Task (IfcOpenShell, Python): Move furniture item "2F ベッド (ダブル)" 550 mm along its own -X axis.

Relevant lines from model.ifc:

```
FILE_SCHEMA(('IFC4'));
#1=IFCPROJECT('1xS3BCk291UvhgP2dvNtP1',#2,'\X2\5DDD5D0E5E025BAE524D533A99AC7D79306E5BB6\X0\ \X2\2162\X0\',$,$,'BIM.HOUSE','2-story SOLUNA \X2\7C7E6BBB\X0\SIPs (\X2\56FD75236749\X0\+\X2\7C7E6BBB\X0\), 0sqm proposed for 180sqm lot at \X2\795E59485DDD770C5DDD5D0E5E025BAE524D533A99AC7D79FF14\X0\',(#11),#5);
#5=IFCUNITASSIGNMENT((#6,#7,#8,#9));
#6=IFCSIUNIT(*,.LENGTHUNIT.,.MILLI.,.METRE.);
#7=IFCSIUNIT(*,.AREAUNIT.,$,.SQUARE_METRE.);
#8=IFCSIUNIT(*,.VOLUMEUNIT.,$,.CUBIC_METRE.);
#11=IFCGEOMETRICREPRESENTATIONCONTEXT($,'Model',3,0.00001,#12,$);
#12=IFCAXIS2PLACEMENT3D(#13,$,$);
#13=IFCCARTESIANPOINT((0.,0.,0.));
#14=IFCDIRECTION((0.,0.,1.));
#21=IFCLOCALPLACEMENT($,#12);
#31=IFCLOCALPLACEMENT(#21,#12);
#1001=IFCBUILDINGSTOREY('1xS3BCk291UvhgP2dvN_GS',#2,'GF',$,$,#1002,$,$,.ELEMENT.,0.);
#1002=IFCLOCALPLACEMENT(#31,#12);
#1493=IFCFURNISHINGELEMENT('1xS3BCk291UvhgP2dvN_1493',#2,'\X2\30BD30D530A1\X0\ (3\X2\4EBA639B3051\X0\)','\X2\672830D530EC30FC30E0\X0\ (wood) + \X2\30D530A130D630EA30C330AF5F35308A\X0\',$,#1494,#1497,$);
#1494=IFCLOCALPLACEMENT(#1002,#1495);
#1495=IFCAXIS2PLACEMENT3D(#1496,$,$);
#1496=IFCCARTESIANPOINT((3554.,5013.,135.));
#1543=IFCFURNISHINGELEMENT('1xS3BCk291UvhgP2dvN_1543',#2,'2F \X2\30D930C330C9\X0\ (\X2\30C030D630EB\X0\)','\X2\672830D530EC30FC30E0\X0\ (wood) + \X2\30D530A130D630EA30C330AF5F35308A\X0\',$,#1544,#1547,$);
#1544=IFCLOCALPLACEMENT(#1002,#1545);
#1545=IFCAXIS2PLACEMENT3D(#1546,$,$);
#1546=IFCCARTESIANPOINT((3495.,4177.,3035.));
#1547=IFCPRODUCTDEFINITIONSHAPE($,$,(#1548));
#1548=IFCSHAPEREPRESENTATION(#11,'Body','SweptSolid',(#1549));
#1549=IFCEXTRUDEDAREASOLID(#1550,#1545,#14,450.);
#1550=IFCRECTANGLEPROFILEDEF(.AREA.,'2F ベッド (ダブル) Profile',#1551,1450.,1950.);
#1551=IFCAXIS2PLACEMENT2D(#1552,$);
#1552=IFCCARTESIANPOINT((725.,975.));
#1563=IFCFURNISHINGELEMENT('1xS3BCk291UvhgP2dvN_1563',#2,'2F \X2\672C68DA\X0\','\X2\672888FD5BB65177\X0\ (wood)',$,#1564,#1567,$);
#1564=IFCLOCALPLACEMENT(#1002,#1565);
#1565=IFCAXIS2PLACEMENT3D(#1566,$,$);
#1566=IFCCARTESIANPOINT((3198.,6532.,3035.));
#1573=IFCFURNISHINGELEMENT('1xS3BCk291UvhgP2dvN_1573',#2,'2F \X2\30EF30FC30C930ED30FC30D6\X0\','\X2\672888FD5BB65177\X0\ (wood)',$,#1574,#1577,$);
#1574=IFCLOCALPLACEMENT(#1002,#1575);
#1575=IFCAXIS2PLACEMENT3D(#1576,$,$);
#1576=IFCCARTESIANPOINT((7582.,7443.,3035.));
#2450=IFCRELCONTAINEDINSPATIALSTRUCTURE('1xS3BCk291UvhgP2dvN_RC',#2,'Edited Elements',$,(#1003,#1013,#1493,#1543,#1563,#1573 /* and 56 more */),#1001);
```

```python
import ifcopenshell
import ifcopenshell.api.geometry
import ifcopenshell.util.placement

model = ifcopenshell.open("model.ifc")

item = model.by_guid("1xS3BCk291UvhgP2dvN_1543")
matrix = ifcopenshell.util.placement.get_local_placement(item.ObjectPlacement)
matrix[:3, 3] -= matrix[:3, 0] * 550.0
ifcopenshell.api.geometry.edit_object_placement(model, product=item, matrix=matrix, is_si=False)

print(ifcopenshell.util.placement.get_local_placement(item.ObjectPlacement).round(3) + 0.0)

model.write("model_rev.ifc")
```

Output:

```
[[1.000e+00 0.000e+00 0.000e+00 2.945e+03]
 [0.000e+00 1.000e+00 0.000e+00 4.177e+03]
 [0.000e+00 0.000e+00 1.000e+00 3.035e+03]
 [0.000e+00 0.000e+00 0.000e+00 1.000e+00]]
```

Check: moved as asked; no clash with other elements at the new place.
